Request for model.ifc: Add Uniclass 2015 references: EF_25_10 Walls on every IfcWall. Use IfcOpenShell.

First a look at what the model holds.

```python
import ifcopenshell

model = ifcopenshell.open("model.ifc")
print(model.schema)
print("classifications:", [c.Name for c in model.by_type("IfcClassification")])
for ifc_class in ("IfcDoor", "IfcRoof", "IfcStair", "IfcWall", "IfcWindow"):
    print(ifc_class, len(model.by_type(ifc_class)))
```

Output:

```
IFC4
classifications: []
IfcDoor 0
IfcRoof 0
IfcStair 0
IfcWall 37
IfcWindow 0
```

```python
import ifcopenshell
import ifcopenshell.api.classification

model = ifcopenshell.open("model.ifc")

system = ifcopenshell.api.classification.add_classification(model, classification="Uniclass 2015")

codes = {
    "IfcWall": ("EF_25_10", "Walls"),
}
for ifc_class, (code, name) in codes.items():
    products = model.by_type(ifc_class)
    ifcopenshell.api.classification.add_reference(
        model, products=products, classification=system, identification=code, name=name
    )
    print(code, len(products))

model.write("model_updated.ifc")
```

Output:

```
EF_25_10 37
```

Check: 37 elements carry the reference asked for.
